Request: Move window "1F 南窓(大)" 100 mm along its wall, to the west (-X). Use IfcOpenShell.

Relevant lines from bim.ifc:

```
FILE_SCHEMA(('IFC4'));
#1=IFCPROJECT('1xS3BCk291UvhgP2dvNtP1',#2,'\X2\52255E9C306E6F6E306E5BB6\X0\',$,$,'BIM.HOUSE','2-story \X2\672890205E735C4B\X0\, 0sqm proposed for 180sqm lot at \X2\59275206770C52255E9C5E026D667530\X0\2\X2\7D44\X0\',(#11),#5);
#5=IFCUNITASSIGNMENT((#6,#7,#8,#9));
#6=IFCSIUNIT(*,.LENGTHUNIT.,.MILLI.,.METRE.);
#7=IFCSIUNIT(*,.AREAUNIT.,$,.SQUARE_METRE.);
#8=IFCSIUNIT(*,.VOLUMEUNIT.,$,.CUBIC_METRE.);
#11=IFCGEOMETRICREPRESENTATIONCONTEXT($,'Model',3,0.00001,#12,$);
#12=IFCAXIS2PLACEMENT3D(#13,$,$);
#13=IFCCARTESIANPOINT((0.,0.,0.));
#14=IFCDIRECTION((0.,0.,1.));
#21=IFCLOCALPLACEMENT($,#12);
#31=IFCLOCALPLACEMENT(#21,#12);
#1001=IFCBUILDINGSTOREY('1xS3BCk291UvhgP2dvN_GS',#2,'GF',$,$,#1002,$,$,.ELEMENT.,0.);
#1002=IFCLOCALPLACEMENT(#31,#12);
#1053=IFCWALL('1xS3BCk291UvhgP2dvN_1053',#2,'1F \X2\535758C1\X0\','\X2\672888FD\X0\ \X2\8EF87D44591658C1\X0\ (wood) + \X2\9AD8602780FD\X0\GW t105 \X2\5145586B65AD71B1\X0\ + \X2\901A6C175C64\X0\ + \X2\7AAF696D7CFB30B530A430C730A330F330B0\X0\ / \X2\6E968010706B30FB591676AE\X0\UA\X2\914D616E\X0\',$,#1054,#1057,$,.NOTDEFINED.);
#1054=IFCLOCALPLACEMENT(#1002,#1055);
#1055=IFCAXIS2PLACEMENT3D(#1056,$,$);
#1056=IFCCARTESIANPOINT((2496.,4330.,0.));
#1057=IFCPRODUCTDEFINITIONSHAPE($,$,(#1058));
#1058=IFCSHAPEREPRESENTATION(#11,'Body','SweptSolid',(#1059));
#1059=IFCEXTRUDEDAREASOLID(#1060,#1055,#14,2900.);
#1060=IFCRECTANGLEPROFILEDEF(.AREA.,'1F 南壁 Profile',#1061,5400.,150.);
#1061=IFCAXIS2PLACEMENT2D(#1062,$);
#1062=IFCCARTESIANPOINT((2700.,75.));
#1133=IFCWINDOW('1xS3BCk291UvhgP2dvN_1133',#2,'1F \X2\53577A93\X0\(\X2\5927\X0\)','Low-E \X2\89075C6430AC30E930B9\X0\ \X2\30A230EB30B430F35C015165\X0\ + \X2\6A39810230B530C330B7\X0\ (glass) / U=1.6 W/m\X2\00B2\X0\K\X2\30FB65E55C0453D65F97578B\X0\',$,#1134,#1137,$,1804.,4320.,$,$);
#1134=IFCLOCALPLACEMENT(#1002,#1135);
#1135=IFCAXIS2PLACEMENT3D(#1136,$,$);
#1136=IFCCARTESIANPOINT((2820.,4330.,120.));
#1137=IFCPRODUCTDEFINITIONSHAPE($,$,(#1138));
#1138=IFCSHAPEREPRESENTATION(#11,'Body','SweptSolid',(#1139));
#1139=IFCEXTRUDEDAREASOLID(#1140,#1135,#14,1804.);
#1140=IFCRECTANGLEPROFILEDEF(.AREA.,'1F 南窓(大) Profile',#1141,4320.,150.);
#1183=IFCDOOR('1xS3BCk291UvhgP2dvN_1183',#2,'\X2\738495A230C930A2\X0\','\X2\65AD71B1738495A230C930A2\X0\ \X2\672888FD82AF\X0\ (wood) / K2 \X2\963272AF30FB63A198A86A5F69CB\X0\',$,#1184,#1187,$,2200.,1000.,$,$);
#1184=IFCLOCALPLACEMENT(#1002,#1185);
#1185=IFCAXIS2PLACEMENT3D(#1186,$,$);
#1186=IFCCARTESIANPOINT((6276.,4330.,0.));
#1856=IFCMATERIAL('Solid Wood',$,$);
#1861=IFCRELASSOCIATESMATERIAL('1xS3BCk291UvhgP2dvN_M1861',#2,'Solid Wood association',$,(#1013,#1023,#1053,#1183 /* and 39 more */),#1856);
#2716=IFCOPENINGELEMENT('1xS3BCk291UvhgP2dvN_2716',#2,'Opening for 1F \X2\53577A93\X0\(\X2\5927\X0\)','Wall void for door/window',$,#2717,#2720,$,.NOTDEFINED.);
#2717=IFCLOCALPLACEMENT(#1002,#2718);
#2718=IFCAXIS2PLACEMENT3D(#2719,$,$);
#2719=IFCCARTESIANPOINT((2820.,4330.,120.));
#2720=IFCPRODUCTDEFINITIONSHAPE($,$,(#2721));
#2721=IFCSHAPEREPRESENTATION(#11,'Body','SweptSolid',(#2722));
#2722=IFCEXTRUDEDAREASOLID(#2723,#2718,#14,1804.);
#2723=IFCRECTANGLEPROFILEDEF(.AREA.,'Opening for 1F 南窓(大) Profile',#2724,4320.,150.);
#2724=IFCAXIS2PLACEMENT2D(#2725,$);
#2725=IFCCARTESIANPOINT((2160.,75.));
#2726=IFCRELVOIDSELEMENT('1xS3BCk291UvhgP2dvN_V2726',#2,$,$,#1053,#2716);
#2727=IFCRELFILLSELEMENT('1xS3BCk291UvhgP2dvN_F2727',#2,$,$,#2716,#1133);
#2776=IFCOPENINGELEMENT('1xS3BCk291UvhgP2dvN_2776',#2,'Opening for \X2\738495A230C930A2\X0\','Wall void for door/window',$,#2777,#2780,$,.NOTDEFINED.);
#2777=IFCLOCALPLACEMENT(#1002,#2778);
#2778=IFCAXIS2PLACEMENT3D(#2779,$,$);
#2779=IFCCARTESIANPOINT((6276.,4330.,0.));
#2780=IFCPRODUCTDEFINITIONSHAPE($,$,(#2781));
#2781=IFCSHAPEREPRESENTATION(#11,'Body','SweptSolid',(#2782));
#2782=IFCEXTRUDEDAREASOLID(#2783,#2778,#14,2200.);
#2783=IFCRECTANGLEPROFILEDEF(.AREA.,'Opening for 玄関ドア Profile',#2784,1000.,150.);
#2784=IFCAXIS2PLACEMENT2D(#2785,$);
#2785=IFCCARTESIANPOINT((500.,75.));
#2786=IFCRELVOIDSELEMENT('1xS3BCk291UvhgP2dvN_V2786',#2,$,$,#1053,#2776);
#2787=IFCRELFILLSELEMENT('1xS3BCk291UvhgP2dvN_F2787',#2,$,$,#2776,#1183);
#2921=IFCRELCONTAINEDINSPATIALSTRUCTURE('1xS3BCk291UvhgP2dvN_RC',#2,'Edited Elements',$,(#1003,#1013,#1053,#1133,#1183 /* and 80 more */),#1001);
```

```python
import ifcopenshell
import ifcopenshell.api.geometry
import ifcopenshell.util.placement

model = ifcopenshell.open("bim.ifc")

window = model.by_id(1133)
opening = window.FillsVoids[0].RelatingOpeningElement
wall = opening.VoidsElements[0].RelatingBuildingElement

wall_matrix = ifcopenshell.util.placement.get_local_placement(wall.ObjectPlacement)
shift = wall_matrix[:3, 0] * -100.0
before = ifcopenshell.util.placement.get_local_placement(window.ObjectPlacement)[:3, 3].copy()

# The window is not placed relative to its opening, so move both.
for product in (opening, window):
    matrix = ifcopenshell.util.placement.get_local_placement(product.ObjectPlacement)
    matrix[:3, 3] += shift
    ifcopenshell.api.geometry.edit_object_placement(model, product=product, matrix=matrix, is_si=False)

after = ifcopenshell.util.placement.get_local_placement(window.ObjectPlacement)[:3, 3]
print("window moved by", (after - before).round(3) + 0.0)

model.write("bim_updated.ifc")
```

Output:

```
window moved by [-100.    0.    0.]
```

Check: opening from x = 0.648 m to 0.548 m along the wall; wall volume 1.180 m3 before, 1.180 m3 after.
